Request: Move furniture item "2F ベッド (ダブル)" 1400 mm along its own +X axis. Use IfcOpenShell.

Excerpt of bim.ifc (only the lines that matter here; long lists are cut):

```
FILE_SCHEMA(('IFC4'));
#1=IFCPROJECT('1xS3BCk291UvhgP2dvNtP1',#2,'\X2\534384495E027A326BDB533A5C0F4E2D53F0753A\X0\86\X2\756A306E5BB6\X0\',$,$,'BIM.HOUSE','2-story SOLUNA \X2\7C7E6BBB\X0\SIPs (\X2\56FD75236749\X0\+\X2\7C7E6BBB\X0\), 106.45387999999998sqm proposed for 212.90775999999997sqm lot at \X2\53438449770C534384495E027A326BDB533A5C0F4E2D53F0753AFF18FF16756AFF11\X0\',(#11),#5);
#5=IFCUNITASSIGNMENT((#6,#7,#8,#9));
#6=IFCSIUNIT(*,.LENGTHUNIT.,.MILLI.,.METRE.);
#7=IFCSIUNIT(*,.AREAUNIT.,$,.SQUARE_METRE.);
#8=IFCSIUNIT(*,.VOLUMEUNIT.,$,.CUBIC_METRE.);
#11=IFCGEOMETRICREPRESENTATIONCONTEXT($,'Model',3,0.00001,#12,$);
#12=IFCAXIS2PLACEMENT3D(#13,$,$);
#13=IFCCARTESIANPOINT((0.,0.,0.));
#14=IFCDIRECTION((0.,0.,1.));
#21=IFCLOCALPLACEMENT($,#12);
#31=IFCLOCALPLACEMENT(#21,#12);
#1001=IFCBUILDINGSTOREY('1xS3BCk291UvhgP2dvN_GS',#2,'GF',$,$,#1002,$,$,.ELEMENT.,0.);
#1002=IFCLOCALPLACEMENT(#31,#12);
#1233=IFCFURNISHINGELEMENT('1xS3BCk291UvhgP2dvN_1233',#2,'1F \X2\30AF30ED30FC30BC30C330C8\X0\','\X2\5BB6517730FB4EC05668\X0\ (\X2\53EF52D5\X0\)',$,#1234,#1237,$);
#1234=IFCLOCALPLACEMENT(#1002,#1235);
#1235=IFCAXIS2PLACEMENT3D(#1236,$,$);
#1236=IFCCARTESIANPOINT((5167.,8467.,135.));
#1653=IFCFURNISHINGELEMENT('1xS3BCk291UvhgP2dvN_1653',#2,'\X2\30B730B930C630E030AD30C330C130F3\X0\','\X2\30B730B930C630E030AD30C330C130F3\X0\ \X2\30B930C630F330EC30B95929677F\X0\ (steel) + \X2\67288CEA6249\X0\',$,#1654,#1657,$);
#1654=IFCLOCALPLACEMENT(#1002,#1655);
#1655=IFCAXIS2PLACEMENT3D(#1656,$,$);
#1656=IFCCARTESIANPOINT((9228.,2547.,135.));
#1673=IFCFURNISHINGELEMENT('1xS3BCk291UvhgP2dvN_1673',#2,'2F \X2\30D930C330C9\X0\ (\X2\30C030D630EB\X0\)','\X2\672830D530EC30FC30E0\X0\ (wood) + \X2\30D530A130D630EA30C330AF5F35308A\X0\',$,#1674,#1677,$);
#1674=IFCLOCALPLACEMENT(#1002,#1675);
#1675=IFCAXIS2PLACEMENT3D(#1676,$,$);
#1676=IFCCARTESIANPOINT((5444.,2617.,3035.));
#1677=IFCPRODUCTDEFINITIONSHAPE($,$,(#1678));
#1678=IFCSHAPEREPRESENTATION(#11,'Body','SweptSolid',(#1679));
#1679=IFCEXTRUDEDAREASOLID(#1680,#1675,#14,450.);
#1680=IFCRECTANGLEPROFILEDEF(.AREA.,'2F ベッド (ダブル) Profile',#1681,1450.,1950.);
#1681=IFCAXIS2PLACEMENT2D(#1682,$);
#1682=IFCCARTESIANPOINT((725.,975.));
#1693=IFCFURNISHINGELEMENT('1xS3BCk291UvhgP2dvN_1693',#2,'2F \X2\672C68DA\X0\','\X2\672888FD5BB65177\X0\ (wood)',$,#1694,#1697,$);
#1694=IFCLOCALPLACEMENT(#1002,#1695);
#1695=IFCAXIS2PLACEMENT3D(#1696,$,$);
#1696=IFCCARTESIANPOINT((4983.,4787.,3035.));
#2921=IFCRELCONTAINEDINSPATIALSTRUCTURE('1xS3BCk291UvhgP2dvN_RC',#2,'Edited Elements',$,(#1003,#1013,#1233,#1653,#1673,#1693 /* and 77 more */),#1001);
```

```python
import ifcopenshell
import ifcopenshell.api.geometry
import ifcopenshell.util.placement
import ifcopenshell.util.unit

model = ifcopenshell.open("bim.ifc")
unit_scale = ifcopenshell.util.unit.calculate_unit_scale(model)

item = model.by_guid("1xS3BCk291UvhgP2dvN_1673")
matrix = ifcopenshell.util.placement.get_local_placement(item.ObjectPlacement)
matrix[:3, 3] += matrix[:3, 0] * 1.4 / unit_scale
ifcopenshell.api.geometry.edit_object_placement(model, product=item, matrix=matrix, is_si=False)

print(ifcopenshell.util.placement.get_local_placement(item.ObjectPlacement).round(3) + 0.0)

model.write("bim-out.ifc")
```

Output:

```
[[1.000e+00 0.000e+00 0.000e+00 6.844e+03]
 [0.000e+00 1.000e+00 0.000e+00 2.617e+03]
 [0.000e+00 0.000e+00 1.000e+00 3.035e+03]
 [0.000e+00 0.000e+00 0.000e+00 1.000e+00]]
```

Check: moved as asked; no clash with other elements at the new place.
